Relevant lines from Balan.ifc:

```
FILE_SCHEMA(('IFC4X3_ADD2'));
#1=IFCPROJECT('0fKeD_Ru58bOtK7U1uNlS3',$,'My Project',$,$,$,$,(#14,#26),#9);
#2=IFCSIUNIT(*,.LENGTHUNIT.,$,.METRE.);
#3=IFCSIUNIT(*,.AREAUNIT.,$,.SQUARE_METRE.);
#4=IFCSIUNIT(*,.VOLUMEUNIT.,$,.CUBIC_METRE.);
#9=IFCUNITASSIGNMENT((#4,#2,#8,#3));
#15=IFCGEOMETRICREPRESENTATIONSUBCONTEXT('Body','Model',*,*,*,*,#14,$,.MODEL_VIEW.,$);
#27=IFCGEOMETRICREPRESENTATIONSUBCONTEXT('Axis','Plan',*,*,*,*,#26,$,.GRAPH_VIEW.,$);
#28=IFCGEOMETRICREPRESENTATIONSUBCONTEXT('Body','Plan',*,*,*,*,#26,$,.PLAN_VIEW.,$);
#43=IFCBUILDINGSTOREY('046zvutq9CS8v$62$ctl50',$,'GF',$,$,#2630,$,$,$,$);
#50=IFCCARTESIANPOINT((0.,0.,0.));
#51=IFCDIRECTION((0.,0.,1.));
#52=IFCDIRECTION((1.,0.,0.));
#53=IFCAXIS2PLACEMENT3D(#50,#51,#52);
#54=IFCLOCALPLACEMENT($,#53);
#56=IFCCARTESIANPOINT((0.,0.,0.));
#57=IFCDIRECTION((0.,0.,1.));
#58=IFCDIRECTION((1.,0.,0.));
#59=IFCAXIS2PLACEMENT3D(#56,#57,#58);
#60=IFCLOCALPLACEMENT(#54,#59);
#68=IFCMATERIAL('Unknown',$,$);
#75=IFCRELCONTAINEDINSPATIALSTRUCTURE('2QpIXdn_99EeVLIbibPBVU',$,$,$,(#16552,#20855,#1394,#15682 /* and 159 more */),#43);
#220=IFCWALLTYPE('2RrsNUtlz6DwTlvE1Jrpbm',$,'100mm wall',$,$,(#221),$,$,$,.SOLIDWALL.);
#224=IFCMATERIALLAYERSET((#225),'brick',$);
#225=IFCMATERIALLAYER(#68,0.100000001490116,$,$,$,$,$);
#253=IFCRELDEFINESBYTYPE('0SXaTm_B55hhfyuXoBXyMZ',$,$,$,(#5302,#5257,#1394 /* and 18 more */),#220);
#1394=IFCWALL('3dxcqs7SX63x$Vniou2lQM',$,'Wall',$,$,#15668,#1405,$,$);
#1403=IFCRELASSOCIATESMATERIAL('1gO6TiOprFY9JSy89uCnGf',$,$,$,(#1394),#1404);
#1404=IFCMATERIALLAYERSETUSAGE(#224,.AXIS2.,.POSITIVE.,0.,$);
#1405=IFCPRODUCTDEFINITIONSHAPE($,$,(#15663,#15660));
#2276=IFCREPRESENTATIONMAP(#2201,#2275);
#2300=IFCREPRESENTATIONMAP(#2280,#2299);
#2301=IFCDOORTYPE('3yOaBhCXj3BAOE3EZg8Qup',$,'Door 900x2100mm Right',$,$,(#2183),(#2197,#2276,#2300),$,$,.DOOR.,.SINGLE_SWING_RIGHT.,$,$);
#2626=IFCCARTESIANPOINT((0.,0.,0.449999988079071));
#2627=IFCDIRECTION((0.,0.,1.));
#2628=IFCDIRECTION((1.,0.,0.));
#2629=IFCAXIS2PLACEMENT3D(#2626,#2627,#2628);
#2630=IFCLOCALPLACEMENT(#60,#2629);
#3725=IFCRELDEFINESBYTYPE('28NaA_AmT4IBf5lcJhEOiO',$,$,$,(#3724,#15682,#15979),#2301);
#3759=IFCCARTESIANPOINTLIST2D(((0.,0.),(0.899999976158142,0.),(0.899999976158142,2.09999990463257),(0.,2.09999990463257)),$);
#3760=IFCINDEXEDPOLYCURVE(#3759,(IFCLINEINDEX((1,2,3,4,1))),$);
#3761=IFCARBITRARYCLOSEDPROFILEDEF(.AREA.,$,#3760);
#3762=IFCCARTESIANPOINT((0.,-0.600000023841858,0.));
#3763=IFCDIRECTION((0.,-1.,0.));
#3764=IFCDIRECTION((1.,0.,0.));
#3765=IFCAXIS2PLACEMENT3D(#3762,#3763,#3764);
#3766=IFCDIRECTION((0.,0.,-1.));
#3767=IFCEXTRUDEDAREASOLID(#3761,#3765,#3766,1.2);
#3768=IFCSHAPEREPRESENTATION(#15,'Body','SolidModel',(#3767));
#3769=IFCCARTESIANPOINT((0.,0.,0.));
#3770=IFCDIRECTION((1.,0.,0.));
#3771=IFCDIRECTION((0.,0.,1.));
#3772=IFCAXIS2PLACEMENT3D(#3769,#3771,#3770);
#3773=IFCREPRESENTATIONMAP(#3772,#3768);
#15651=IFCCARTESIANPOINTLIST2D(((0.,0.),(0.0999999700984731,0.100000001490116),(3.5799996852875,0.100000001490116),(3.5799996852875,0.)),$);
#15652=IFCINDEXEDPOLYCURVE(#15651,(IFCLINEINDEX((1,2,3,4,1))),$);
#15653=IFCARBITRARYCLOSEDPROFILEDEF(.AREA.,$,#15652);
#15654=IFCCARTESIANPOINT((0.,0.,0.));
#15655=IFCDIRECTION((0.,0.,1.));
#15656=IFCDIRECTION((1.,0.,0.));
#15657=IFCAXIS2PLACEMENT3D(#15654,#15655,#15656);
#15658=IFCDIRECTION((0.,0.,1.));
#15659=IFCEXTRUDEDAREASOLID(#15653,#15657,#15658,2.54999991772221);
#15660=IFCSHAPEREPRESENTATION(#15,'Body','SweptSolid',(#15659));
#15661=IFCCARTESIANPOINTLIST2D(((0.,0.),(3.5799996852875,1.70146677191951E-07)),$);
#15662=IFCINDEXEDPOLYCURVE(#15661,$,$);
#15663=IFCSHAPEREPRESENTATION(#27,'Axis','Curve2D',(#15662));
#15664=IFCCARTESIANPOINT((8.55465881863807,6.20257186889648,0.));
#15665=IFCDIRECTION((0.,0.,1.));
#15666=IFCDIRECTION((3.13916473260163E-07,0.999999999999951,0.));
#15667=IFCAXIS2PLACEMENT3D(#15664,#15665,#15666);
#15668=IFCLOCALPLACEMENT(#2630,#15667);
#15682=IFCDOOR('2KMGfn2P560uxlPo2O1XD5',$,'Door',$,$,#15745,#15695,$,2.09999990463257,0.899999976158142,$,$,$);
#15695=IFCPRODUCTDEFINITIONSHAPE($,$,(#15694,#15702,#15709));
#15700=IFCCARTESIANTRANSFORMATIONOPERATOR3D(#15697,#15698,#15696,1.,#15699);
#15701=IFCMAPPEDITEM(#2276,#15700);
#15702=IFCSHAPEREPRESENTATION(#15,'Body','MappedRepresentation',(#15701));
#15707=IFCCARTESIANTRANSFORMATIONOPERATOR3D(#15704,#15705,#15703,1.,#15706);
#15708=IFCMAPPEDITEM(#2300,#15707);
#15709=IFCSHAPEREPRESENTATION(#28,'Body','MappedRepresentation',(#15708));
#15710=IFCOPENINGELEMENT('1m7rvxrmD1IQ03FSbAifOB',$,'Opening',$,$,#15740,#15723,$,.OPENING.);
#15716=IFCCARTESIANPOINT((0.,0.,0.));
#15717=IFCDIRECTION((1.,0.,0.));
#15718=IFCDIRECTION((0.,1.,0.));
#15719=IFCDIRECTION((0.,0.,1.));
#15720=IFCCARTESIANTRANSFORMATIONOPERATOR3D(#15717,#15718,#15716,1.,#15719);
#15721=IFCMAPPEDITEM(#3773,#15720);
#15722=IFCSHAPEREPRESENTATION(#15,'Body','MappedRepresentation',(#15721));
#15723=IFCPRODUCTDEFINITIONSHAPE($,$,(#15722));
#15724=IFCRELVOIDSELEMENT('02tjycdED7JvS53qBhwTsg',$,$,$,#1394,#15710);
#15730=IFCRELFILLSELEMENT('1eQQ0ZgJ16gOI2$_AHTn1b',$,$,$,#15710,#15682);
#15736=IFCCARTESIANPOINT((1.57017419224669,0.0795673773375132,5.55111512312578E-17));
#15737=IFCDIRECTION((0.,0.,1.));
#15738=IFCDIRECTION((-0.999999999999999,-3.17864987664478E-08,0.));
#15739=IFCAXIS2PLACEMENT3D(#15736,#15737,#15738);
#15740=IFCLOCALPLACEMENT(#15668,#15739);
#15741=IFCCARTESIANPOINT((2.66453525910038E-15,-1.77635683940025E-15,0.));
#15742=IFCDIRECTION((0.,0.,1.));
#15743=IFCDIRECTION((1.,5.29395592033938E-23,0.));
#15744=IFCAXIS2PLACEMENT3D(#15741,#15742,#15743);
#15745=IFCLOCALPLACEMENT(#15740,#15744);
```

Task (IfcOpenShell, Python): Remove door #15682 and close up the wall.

```python
import ifcopenshell
import ifcopenshell.api.feature
import ifcopenshell.api.root
import ifcopenshell.geom
import ifcopenshell.util.shape

model = ifcopenshell.open("Balan.ifc")
settings = ifcopenshell.geom.settings()


def volume(element):
    """Net volume in cubic metres, openings subtracted."""
    shape = ifcopenshell.geom.create_shape(settings, element)
    return ifcopenshell.util.shape.get_volume(shape.geometry)


door = model.by_guid("2KMGfn2P560uxlPo2O1XD5")
opening = door.FillsVoids[0].RelatingOpeningElement
wall = opening.VoidsElements[0].RelatingBuildingElement
before = volume(wall)

ifcopenshell.api.root.remove_product(model, product=door)
ifcopenshell.api.feature.remove_feature(model, feature=opening)

after = volume(wall)

print(f"wall volume {before:.3f} -> {after:.3f} m3")

model.write("Balan_v2.ifc")
```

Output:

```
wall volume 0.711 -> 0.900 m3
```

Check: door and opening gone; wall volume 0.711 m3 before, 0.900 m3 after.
